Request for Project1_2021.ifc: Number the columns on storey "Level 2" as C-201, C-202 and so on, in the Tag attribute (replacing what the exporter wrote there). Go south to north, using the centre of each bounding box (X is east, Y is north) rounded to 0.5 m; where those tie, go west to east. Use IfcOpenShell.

First a look at what the model holds.

```python
import ifcopenshell
import ifcopenshell.util.element
import ifcopenshell.util.placement

model = ifcopenshell.open("Project1_2021.ifc")
print(model.schema)
storey = next(s for s in model.by_type("IfcBuildingStorey") if s.Name == "Level 2")
columns = [e for e in ifcopenshell.util.element.get_decomposition(storey) if e.is_a("IfcColumn")]
for e in sorted(columns, key=lambda e: e.id()):
    origin = ifcopenshell.util.placement.get_local_placement(e.ObjectPlacement)[:3, 3]
    print(e.id(), e.Tag, e.Name, origin.round(2) + 0.0, sep=" | ")
```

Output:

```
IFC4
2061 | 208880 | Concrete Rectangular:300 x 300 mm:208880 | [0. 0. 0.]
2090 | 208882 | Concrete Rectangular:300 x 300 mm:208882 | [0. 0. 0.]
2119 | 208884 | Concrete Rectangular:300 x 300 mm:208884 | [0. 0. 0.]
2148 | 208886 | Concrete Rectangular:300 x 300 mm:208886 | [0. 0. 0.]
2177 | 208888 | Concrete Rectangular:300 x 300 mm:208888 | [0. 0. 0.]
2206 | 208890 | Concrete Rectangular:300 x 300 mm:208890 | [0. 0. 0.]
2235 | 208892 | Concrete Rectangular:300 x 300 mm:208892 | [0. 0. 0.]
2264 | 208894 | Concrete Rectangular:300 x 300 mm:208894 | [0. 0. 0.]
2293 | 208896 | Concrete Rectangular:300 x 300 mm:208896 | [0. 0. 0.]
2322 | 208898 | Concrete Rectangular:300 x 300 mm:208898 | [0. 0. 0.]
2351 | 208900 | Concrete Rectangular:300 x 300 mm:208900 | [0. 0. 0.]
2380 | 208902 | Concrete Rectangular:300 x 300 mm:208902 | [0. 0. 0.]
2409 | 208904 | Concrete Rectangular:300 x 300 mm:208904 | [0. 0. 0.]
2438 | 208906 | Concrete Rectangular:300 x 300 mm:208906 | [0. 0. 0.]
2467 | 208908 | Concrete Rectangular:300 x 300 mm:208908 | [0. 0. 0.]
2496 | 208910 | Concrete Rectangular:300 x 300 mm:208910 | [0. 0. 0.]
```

```python
import ifcopenshell
import ifcopenshell.geom
import ifcopenshell.util.element
import ifcopenshell.util.shape

model = ifcopenshell.open("Project1_2021.ifc")
settings = ifcopenshell.geom.settings()
settings.set("use-world-coords", True)


def centre(element):
    shape = ifcopenshell.geom.create_shape(settings, element)
    return ifcopenshell.util.shape.get_bbox_centroid(shape.geometry)


storey = next(s for s in model.by_type("IfcBuildingStorey") if s.Name == "Level 2")
columns = [e for e in ifcopenshell.util.element.get_decomposition(storey) if e.is_a("IfcColumn")]

# Insertion points can sit at a corner or the storey origin, so sort by the geometry (in metres).
centres = {e: centre(e) for e in columns}
columns.sort(key=lambda e: (round(centres[e][1] / 0.5), centres[e][0]))

for i, e in enumerate(columns, start=1):
    number = f"C-2{i:02d}"
    e.Tag = number
    print(e.id(), number)

model.write("Project1_2021_updated.ifc")
```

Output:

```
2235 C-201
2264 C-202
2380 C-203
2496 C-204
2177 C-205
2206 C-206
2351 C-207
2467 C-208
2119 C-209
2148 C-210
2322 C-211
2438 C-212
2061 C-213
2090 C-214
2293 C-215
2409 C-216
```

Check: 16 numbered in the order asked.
